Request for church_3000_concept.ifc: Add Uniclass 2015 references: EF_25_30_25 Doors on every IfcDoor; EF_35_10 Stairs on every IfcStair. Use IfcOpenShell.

First a look at what the model holds.

```python
import ifcopenshell

model = ifcopenshell.open("church_3000_concept.ifc")
print(model.schema)
print("classifications:", [c.Name for c in model.by_type("IfcClassification")])
for ifc_class in ("IfcDoor", "IfcRoof", "IfcStair", "IfcWall", "IfcWindow"):
    print(ifc_class, len(model.by_type(ifc_class)))
```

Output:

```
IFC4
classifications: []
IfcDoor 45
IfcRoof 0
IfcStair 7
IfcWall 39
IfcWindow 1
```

```python
import ifcopenshell
import ifcopenshell.api.classification

model = ifcopenshell.open("church_3000_concept.ifc")

system = ifcopenshell.api.classification.add_classification(model, classification="Uniclass 2015")

codes = {
    "IfcDoor": ("EF_25_30_25", "Doors"),
    "IfcStair": ("EF_35_10", "Stairs"),
}
for ifc_class, (code, name) in codes.items():
    products = model.by_type(ifc_class)
    ifcopenshell.api.classification.add_reference(
        model, products=products, classification=system, identification=code, name=name
    )
    print(code, len(products))

model.write("church_3000_concept-out.ifc")
```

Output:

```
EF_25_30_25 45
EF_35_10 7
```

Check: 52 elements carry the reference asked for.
